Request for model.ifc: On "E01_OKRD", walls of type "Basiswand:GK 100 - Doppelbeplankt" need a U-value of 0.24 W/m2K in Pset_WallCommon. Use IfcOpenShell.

First a look at what the model holds.

```python
import ifcopenshell
import ifcopenshell.util.element

model = ifcopenshell.open("model.ifc")
print(model.schema)
storey = next(s for s in model.by_type("IfcBuildingStorey") if s.Name == "E01_OKRD")
walls = [e for e in ifcopenshell.util.element.get_decomposition(storey) if e.is_a("IfcWall")]
seen = {}
for e in walls:
    element_type = ifcopenshell.util.element.get_type(e)
    key = (element_type.Name if element_type != e and element_type else None, ifcopenshell.util.element.get_pset(e, "Pset_WallCommon", "ThermalTransmittance"))
    seen[key] = seen.get(key, 0) + 1
for (name, value), count in sorted(seen.items(), key=str):
    print(count, "x", name, "|", value)
```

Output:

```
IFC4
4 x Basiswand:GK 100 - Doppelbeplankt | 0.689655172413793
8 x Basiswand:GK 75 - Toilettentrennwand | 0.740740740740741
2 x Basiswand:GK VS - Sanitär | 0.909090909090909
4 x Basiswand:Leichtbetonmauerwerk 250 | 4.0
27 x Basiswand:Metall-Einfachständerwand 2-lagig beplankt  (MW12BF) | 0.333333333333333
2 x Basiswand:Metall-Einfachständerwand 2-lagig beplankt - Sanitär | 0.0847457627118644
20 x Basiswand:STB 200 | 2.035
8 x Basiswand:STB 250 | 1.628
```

```python
import ifcopenshell
import ifcopenshell.api.pset
import ifcopenshell.util.element

model = ifcopenshell.open("model.ifc")

storey = next(s for s in model.by_type("IfcBuildingStorey") if s.Name == "E01_OKRD")
walls = [e for e in ifcopenshell.util.element.get_decomposition(storey) if e.is_a("IfcWall")]

count = 0
for e in walls:
    element_type = ifcopenshell.util.element.get_type(e)
    if element_type in (None, e) or element_type.Name != "Basiswand:GK 100 - Doppelbeplankt":
        continue
    # add_pset returns the element's existing set when there is one.
    pset = ifcopenshell.api.pset.add_pset(model, product=e, name="Pset_WallCommon")
    ifcopenshell.api.pset.edit_pset(model, pset=pset, properties={"ThermalTransmittance": 0.24})
    count += 1

print(count, "walls updated")

model.write("model_rev.ifc")
```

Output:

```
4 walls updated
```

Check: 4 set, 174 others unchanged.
